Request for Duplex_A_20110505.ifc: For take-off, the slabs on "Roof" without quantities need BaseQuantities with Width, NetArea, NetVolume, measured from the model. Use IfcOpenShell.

First a look at what the model holds.

```python
import ifcopenshell
import ifcopenshell.util.element
import ifcopenshell.util.unit

model = ifcopenshell.open("Duplex_A_20110505.ifc")
print(model.schema)
for unit_type in ("LENGTHUNIT", "AREAUNIT", "VOLUMEUNIT"):
    print(unit_type, ifcopenshell.util.unit.calculate_unit_scale(model, unit_type))
storey = next(s for s in model.by_type("IfcBuildingStorey") if s.Name == "Roof")
slabs = [e for e in ifcopenshell.util.element.get_decomposition(storey) if e.is_a("IfcSlab")]
for e in sorted(slabs, key=lambda e: e.id()):
    print(e.id(), e.is_a(), e.Name, list(ifcopenshell.util.element.get_psets(e, qtos_only=True)), sep=" | ")
```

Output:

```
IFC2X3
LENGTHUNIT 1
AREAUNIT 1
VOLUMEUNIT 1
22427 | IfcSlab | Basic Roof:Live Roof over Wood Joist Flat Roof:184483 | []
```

```python
import ifcopenshell
import ifcopenshell.api.pset
import ifcopenshell.geom
import ifcopenshell.util.element
import ifcopenshell.util.shape
import ifcopenshell.util.unit

model = ifcopenshell.open("Duplex_A_20110505.ifc")
unit_scale = ifcopenshell.util.unit.calculate_unit_scale(model)
area_scale = ifcopenshell.util.unit.calculate_unit_scale(model, "AREAUNIT")
volume_scale = ifcopenshell.util.unit.calculate_unit_scale(model, "VOLUMEUNIT")
settings = ifcopenshell.geom.settings()

storey = next(s for s in model.by_type("IfcBuildingStorey") if s.Name == "Roof")
slabs = [e for e in ifcopenshell.util.element.get_decomposition(storey) if e.is_a("IfcSlab")]

for e in sorted(slabs, key=lambda e: e.id()):
    if ifcopenshell.util.element.get_psets(e, qtos_only=True, should_inherit=False):
        continue
    # Geometry comes back in metres, in the element's own axes.
    shape = ifcopenshell.geom.create_shape(settings, e)
    values = {
        "Width": ifcopenshell.util.shape.get_z(shape.geometry) / unit_scale,
        "NetArea": ifcopenshell.util.shape.get_footprint_area(shape.geometry) / area_scale,
        "NetVolume": ifcopenshell.util.shape.get_volume(shape.geometry) / volume_scale,
    }
    qto = ifcopenshell.api.pset.add_qto(model, product=e, name="BaseQuantities")
    ifcopenshell.api.pset.edit_qto(model, qto=qto, properties=values)
    print(e.id(), {k: round(v, 3) for k, v in values.items()})

model.write("Duplex_A_20110505_v2.ifc")
```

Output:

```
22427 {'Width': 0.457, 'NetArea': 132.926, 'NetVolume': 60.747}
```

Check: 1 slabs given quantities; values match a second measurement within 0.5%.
